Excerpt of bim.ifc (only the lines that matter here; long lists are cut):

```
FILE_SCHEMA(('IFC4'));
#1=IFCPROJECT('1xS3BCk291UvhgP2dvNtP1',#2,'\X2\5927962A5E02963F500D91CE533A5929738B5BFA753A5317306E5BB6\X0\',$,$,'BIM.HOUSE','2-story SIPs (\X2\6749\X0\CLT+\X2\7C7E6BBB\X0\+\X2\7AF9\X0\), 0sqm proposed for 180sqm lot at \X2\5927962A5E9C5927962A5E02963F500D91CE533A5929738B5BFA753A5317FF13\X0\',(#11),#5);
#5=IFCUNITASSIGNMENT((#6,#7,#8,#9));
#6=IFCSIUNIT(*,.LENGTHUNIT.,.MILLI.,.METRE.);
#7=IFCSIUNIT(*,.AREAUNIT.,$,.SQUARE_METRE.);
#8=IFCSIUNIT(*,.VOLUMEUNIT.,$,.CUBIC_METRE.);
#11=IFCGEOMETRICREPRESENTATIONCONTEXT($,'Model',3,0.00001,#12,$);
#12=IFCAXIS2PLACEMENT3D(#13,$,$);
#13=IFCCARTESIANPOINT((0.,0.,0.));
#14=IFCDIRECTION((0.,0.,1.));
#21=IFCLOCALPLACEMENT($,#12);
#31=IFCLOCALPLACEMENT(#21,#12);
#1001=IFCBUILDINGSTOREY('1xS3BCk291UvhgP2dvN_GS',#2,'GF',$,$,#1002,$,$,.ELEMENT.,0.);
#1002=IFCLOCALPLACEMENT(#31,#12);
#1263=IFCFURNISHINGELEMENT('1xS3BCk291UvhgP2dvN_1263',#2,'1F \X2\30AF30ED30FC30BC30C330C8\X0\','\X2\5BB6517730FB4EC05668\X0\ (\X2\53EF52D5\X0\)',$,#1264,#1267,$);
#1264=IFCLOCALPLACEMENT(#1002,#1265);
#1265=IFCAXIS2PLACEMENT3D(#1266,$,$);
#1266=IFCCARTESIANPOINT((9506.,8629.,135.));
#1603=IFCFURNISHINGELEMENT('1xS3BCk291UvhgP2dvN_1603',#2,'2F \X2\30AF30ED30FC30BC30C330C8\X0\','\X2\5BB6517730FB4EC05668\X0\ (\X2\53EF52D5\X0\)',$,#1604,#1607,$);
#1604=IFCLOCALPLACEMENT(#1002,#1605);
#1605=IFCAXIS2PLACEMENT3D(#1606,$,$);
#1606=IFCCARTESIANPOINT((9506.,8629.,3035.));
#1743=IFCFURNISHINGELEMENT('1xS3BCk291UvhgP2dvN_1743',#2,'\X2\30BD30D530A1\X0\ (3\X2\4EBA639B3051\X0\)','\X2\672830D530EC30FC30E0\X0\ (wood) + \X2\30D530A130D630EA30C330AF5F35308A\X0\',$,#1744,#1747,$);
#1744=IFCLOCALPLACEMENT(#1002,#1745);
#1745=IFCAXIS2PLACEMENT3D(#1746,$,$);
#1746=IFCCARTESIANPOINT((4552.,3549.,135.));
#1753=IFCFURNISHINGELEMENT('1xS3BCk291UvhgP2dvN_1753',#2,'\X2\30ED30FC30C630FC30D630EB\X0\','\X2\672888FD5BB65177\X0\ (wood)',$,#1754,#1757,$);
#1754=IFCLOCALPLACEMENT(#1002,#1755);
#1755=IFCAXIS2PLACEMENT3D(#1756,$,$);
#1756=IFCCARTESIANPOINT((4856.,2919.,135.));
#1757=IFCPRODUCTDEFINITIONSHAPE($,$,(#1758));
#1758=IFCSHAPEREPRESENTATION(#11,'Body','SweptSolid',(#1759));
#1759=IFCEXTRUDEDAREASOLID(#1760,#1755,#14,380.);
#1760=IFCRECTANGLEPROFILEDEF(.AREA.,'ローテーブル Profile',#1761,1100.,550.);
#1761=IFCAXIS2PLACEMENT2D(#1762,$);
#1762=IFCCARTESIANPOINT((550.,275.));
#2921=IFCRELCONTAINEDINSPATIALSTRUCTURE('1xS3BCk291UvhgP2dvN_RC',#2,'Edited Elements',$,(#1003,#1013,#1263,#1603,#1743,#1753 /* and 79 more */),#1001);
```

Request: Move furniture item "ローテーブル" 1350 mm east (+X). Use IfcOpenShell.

```python
import ifcopenshell
import ifcopenshell.api.geometry
import ifcopenshell.util.placement
import ifcopenshell.util.unit

model = ifcopenshell.open("bim.ifc")
unit_scale = ifcopenshell.util.unit.calculate_unit_scale(model)

item = model.by_guid("1xS3BCk291UvhgP2dvN_1753")
matrix = ifcopenshell.util.placement.get_local_placement(item.ObjectPlacement)
matrix[0, 3] += 1.35 / unit_scale
ifcopenshell.api.geometry.edit_object_placement(model, product=item, matrix=matrix, is_si=False)

print(ifcopenshell.util.placement.get_local_placement(item.ObjectPlacement).round(3) + 0.0)

model.write("bim_updated.ifc")
```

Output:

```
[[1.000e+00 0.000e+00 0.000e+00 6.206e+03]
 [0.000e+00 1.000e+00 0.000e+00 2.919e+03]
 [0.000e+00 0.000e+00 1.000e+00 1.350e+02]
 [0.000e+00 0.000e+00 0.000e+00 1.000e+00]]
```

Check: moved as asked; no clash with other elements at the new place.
